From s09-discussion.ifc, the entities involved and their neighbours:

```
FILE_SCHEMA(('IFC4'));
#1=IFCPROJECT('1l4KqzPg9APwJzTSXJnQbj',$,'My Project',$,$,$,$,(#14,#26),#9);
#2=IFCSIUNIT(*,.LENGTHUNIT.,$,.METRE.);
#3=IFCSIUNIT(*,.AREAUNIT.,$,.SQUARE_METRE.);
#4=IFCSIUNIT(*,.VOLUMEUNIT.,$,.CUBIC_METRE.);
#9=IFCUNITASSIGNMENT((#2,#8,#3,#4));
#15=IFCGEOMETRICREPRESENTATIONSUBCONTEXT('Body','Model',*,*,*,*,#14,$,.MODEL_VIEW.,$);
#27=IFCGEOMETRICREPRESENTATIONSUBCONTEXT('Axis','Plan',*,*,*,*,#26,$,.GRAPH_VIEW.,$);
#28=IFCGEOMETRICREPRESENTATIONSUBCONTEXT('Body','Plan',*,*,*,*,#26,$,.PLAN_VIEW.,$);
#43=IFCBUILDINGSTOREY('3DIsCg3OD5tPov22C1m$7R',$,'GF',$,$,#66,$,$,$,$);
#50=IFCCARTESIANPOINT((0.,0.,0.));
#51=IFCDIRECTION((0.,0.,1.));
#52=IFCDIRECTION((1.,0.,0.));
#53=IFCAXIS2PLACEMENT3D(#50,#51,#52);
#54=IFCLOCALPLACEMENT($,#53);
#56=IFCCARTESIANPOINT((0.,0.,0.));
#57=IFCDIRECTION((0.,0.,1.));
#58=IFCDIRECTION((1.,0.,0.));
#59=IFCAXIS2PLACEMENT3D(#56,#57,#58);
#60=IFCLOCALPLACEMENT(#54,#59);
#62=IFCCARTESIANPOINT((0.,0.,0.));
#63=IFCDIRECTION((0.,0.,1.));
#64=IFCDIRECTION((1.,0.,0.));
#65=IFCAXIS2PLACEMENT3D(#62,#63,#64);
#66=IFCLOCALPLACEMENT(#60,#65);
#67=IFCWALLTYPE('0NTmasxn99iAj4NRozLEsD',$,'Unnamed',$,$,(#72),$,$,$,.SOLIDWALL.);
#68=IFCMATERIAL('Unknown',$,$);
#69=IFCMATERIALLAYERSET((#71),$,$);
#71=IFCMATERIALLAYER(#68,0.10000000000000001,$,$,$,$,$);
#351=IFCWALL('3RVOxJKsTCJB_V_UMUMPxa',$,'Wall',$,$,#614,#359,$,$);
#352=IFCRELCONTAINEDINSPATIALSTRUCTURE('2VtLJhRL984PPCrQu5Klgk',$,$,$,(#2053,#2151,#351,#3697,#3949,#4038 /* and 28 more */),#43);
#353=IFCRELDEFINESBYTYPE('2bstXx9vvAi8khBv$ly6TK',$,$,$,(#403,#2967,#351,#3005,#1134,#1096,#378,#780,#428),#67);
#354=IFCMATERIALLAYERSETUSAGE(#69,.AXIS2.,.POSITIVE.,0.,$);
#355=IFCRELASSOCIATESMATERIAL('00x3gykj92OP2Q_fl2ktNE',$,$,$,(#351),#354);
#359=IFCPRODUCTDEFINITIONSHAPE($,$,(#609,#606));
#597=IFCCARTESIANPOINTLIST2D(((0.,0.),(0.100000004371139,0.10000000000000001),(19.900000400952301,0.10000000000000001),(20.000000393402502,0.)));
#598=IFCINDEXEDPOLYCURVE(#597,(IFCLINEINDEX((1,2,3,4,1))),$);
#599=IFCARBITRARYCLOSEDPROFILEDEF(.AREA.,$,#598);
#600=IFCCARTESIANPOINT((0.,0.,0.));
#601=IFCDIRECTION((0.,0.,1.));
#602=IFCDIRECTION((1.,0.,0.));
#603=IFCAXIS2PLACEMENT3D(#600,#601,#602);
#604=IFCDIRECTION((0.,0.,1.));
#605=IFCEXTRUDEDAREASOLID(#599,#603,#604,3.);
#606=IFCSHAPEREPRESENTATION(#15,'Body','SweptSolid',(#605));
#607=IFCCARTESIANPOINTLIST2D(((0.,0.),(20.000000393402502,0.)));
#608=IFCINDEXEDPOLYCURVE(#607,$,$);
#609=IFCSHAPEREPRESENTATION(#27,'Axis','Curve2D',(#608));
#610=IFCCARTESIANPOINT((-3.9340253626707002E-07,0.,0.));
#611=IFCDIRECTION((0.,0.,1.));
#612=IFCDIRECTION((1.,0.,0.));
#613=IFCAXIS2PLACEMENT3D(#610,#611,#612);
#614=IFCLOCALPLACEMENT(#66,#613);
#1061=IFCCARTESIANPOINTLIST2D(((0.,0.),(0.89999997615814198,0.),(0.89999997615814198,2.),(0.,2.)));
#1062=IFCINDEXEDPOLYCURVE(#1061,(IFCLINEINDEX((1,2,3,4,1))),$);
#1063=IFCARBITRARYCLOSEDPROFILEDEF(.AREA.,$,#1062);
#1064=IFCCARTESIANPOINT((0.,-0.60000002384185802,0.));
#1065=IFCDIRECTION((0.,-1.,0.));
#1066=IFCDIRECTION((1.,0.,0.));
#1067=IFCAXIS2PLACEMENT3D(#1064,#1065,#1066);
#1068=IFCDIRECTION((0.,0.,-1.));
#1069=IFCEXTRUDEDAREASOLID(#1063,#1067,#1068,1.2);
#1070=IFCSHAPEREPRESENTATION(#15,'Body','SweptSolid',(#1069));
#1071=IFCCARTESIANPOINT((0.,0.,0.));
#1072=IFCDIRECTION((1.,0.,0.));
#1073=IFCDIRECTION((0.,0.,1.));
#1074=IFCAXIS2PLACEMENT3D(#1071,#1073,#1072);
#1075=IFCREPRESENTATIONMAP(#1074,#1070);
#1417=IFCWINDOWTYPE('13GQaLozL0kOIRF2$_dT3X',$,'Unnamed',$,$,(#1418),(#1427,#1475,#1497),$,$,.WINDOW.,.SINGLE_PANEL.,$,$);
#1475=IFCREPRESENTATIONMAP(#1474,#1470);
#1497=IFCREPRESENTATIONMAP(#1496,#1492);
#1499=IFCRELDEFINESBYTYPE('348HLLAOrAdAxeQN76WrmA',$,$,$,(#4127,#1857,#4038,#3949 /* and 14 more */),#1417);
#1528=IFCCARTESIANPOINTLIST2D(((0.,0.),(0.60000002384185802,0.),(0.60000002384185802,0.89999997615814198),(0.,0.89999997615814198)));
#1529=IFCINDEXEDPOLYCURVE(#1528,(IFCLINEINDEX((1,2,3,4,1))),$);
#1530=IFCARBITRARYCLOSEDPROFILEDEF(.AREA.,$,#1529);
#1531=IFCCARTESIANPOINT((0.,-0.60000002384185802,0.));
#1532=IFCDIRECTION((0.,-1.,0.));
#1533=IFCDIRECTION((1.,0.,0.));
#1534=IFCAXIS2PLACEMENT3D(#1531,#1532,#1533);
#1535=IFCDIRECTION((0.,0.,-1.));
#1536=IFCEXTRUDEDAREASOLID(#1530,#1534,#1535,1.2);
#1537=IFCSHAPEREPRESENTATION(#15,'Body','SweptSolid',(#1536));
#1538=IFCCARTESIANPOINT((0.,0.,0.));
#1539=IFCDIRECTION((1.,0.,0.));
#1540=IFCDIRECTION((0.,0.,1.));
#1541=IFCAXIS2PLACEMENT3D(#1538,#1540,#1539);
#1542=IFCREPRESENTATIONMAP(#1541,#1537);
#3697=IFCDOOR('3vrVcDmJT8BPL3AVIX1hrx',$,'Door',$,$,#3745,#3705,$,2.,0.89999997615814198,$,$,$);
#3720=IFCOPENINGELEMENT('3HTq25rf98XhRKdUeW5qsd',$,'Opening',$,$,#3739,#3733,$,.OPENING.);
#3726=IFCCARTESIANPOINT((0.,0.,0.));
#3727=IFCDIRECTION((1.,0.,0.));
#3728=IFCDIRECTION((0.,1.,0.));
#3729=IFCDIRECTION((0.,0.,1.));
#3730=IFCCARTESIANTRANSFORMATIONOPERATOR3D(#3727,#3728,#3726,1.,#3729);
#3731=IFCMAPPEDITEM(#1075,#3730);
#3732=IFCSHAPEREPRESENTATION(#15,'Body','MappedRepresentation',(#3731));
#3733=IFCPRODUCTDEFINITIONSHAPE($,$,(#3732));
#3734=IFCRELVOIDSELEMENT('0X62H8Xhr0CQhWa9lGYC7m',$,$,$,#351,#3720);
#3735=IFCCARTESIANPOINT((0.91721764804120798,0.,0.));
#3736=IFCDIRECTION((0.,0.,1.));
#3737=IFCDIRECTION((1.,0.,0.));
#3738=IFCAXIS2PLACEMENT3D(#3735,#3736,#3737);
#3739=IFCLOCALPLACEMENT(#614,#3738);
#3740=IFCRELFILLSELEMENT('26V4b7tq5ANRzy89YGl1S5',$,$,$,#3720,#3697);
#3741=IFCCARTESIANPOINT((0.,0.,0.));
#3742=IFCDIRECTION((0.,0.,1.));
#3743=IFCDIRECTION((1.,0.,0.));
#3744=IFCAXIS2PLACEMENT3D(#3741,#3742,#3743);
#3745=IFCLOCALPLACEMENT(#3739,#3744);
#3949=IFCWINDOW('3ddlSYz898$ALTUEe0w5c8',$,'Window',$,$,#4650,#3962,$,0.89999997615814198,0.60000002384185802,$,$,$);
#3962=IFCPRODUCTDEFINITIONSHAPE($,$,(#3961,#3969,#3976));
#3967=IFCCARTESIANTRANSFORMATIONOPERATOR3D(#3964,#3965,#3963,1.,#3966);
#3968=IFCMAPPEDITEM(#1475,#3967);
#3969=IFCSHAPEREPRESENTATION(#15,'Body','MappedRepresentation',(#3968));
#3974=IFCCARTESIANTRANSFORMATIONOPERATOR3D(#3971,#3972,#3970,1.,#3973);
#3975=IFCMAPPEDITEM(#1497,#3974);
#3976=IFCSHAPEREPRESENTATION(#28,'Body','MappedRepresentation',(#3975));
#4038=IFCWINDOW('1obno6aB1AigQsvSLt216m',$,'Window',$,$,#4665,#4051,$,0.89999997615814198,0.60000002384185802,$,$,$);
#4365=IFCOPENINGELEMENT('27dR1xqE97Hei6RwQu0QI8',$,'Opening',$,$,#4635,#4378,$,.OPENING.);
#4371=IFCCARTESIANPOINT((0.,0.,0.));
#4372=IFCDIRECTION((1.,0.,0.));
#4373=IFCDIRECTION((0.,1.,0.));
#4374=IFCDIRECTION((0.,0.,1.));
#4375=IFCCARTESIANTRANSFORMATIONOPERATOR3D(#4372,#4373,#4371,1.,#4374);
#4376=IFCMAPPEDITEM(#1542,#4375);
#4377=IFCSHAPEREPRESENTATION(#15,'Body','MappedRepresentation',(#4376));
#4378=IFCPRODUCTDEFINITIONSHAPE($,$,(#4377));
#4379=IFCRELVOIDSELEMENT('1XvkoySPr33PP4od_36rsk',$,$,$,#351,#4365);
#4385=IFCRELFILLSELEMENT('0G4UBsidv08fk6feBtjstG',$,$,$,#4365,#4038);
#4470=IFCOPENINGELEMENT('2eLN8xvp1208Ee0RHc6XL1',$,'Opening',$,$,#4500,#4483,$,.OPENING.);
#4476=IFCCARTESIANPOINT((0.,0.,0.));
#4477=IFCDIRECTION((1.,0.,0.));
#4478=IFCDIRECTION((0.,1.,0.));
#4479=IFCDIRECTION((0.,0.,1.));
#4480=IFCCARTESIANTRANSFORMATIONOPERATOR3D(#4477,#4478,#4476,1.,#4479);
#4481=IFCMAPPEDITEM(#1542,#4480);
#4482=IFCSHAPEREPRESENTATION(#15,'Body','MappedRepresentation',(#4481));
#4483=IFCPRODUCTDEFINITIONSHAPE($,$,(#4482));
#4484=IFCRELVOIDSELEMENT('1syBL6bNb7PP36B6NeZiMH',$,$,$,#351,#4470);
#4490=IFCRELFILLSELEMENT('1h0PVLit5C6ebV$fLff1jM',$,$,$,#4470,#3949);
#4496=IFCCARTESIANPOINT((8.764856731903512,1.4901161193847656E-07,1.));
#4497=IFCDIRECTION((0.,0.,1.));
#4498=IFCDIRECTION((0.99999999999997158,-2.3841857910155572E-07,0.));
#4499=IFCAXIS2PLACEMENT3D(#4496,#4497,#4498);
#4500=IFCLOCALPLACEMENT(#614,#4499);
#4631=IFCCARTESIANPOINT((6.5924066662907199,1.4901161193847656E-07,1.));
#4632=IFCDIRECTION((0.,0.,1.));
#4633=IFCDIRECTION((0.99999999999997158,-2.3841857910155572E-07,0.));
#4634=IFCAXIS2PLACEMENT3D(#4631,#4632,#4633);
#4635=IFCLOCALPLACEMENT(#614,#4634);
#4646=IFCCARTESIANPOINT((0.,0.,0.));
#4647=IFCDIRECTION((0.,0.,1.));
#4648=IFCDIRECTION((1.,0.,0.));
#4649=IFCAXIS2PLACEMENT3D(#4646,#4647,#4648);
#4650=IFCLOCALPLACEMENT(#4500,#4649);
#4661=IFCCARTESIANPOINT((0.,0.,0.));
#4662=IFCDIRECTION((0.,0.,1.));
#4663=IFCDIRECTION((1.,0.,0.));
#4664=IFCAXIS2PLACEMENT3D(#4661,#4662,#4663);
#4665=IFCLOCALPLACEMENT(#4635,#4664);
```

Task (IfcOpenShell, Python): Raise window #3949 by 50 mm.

```python
import numpy as np
import ifcopenshell
import ifcopenshell.api.geometry
import ifcopenshell.util.placement
import ifcopenshell.util.unit

model = ifcopenshell.open("s09-discussion.ifc")
unit_scale = ifcopenshell.util.unit.calculate_unit_scale(model)

window = model.by_id(3949)
opening = window.FillsVoids[0].RelatingOpeningElement
dz = 0.05 / unit_scale

shift = np.array([0.0, 0.0, dz])
# The window is placed relative to its opening, so it follows when the opening moves.
matrix = ifcopenshell.util.placement.get_local_placement(opening.ObjectPlacement)
matrix[:3, 3] += shift
ifcopenshell.api.geometry.edit_object_placement(
    model, product=opening, matrix=matrix, is_si=False, should_transform_children=True
)

print(f"moved by {dz * unit_scale:+.3f} m")

model.write("s09-discussion_updated.ifc")
```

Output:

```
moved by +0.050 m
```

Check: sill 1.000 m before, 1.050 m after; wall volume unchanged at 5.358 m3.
